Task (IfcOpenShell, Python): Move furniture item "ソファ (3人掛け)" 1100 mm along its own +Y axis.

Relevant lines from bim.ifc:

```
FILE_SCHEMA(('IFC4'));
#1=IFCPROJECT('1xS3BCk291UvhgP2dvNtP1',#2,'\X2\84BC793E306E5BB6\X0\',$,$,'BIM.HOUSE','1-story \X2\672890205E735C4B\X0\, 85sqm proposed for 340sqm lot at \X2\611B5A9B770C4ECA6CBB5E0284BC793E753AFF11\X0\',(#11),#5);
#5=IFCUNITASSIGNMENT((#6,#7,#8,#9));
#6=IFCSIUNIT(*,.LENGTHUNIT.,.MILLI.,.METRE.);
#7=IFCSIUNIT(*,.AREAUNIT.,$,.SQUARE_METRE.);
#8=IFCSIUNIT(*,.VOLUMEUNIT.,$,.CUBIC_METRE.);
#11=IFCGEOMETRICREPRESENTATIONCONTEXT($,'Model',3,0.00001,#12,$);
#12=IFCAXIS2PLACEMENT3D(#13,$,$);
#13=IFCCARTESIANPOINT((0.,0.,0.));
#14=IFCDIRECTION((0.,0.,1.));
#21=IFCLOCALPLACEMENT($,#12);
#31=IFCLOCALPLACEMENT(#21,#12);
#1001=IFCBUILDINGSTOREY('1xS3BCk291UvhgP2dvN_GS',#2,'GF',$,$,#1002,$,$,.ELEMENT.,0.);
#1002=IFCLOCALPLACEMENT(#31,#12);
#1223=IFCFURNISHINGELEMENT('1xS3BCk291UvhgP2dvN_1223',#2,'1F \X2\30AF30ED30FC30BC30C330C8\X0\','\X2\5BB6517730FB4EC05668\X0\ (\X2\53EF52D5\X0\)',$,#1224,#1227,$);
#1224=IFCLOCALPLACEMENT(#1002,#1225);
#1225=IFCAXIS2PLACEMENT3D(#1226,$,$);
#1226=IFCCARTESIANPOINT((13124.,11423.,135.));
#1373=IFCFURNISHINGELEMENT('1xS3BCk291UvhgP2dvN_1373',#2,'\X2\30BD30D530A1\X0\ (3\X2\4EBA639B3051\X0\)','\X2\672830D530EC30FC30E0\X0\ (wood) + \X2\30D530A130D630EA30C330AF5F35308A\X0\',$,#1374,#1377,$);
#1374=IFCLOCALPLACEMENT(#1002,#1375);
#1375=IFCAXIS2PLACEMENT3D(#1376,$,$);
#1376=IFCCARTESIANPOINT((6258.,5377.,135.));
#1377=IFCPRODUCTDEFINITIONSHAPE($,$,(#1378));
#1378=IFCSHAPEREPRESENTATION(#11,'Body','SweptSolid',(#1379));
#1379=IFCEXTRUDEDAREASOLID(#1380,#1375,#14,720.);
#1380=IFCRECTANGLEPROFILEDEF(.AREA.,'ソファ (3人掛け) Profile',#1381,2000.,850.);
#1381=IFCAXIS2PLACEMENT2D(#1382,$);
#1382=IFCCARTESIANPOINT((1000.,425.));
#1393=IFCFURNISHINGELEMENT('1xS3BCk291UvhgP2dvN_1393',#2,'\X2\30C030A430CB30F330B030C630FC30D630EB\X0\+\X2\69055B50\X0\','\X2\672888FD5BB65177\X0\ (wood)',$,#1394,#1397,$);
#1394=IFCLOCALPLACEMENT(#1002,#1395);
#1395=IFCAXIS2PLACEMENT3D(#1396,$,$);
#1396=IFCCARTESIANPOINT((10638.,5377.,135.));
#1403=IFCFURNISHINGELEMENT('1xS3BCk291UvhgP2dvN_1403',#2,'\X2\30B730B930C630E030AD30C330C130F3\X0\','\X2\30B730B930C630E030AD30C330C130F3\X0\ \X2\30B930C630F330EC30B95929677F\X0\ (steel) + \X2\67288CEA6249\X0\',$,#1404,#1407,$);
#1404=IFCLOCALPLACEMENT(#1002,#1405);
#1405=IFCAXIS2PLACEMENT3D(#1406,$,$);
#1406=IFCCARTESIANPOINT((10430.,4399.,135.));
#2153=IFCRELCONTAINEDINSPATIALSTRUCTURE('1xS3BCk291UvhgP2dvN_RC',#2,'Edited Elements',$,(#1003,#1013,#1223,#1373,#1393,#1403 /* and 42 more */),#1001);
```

```python
import ifcopenshell
import ifcopenshell.api.geometry
import ifcopenshell.util.placement
import ifcopenshell.util.unit

model = ifcopenshell.open("bim.ifc")
unit_scale = ifcopenshell.util.unit.calculate_unit_scale(model)

item = model.by_guid("1xS3BCk291UvhgP2dvN_1373")
matrix = ifcopenshell.util.placement.get_local_placement(item.ObjectPlacement)
matrix[:3, 3] += matrix[:3, 1] * 1.1 / unit_scale
ifcopenshell.api.geometry.edit_object_placement(model, product=item, matrix=matrix, is_si=False)

print(ifcopenshell.util.placement.get_local_placement(item.ObjectPlacement).round(3) + 0.0)

model.write("bim_edited.ifc")
```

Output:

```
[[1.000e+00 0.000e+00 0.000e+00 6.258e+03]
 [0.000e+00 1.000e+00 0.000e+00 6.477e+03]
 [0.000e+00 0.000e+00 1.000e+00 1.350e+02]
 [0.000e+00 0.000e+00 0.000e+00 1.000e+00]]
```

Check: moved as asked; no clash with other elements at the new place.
